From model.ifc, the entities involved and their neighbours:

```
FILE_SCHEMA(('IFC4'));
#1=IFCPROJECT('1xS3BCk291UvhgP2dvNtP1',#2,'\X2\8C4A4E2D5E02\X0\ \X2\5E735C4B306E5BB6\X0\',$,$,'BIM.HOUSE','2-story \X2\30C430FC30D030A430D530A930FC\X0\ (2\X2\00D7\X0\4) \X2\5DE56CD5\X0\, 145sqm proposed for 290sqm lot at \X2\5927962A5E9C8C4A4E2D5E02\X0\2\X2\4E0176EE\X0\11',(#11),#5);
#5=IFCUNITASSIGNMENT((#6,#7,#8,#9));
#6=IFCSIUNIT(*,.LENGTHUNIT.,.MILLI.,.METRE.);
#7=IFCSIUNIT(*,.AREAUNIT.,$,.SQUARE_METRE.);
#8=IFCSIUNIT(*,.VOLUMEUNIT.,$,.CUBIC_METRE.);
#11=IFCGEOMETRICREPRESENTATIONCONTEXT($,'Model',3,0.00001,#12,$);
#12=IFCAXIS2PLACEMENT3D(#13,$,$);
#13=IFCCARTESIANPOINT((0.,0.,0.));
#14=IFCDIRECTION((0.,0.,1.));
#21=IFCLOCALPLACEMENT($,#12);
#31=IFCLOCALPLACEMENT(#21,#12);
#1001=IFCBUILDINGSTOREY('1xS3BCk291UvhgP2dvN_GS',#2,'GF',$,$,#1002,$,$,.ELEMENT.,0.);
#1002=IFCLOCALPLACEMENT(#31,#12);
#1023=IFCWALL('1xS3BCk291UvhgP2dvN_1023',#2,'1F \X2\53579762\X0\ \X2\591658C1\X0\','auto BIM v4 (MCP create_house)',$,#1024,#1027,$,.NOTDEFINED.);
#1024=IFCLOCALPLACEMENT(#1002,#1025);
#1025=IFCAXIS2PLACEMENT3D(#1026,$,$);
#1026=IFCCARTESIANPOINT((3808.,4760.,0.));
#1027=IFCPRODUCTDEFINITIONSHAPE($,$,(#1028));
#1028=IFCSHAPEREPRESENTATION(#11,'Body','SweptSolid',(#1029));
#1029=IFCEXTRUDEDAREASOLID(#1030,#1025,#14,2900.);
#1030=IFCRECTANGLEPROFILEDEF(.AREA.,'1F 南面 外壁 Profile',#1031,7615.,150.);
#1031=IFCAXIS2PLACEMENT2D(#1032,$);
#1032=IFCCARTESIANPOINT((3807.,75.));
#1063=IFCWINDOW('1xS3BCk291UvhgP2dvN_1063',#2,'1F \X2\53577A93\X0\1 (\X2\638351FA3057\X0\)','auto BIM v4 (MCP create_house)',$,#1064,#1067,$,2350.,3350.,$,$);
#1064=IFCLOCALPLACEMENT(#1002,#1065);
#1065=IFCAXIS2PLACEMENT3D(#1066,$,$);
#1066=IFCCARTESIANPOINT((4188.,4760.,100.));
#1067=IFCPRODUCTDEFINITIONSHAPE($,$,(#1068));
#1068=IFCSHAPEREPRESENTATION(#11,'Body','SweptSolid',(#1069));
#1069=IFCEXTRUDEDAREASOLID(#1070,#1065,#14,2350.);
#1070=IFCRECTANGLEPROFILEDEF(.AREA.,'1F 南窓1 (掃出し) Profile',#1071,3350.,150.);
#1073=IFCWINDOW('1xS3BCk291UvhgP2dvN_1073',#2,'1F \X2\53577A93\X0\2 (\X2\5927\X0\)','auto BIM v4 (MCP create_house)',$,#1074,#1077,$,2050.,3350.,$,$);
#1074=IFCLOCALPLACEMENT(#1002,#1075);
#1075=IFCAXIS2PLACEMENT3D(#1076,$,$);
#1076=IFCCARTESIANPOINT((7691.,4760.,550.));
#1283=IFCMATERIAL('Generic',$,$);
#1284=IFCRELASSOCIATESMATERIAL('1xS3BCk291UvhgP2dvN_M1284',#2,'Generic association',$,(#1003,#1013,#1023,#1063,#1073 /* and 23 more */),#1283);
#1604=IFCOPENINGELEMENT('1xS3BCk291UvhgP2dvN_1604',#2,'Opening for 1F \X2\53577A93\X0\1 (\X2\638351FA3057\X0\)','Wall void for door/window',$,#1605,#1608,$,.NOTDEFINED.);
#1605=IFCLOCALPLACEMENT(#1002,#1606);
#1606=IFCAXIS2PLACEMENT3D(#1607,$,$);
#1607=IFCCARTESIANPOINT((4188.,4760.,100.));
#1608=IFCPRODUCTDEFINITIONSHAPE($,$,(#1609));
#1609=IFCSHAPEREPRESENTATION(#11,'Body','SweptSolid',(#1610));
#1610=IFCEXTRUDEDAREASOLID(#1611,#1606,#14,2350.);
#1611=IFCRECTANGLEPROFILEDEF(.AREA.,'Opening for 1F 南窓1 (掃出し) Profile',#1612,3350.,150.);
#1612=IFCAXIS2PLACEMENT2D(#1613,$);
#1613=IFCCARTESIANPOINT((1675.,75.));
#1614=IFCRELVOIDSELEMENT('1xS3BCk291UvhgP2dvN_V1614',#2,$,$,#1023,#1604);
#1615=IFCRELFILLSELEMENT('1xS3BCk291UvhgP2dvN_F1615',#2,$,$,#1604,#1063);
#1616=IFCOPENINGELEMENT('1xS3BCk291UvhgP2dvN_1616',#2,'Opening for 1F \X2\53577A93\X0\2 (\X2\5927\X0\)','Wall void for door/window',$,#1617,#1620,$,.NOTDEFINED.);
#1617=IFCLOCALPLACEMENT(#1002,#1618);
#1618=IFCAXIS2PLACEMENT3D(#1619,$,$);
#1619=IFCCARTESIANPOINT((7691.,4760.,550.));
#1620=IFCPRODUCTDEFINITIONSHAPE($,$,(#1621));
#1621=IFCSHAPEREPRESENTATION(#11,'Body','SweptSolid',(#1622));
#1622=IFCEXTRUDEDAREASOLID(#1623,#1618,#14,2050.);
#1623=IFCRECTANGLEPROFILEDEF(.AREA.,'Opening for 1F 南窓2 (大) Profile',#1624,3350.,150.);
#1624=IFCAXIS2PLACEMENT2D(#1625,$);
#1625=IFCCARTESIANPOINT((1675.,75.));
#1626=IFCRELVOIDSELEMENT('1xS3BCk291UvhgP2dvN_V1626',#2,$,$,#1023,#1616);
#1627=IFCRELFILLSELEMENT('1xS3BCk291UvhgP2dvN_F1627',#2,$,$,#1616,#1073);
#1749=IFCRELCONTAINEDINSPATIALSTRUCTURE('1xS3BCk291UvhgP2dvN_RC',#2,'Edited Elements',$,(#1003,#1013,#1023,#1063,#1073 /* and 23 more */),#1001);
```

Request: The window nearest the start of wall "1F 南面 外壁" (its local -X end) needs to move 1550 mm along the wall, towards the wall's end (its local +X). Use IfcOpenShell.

```python
import ifcopenshell
import ifcopenshell.api.geometry
import ifcopenshell.util.placement
import ifcopenshell.util.unit

model = ifcopenshell.open("model.ifc")
unit_scale = ifcopenshell.util.unit.calculate_unit_scale(model)

window = model.by_guid("1xS3BCk291UvhgP2dvN_1063")
opening = window.FillsVoids[0].RelatingOpeningElement
wall = opening.VoidsElements[0].RelatingBuildingElement

wall_matrix = ifcopenshell.util.placement.get_local_placement(wall.ObjectPlacement)
shift = wall_matrix[:3, 0] * 1.55 / unit_scale
before = ifcopenshell.util.placement.get_local_placement(window.ObjectPlacement)[:3, 3].copy()

# The window is not placed relative to its opening, so move both.
for product in (opening, window):
    matrix = ifcopenshell.util.placement.get_local_placement(product.ObjectPlacement)
    matrix[:3, 3] += shift
    ifcopenshell.api.geometry.edit_object_placement(model, product=product, matrix=matrix, is_si=False)

after = ifcopenshell.util.placement.get_local_placement(window.ObjectPlacement)[:3, 3]
print("window moved by", (after - before).round(3) + 0.0)

model.write("model-out.ifc")
```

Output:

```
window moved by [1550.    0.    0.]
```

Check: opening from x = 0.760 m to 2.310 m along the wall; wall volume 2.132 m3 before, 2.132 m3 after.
